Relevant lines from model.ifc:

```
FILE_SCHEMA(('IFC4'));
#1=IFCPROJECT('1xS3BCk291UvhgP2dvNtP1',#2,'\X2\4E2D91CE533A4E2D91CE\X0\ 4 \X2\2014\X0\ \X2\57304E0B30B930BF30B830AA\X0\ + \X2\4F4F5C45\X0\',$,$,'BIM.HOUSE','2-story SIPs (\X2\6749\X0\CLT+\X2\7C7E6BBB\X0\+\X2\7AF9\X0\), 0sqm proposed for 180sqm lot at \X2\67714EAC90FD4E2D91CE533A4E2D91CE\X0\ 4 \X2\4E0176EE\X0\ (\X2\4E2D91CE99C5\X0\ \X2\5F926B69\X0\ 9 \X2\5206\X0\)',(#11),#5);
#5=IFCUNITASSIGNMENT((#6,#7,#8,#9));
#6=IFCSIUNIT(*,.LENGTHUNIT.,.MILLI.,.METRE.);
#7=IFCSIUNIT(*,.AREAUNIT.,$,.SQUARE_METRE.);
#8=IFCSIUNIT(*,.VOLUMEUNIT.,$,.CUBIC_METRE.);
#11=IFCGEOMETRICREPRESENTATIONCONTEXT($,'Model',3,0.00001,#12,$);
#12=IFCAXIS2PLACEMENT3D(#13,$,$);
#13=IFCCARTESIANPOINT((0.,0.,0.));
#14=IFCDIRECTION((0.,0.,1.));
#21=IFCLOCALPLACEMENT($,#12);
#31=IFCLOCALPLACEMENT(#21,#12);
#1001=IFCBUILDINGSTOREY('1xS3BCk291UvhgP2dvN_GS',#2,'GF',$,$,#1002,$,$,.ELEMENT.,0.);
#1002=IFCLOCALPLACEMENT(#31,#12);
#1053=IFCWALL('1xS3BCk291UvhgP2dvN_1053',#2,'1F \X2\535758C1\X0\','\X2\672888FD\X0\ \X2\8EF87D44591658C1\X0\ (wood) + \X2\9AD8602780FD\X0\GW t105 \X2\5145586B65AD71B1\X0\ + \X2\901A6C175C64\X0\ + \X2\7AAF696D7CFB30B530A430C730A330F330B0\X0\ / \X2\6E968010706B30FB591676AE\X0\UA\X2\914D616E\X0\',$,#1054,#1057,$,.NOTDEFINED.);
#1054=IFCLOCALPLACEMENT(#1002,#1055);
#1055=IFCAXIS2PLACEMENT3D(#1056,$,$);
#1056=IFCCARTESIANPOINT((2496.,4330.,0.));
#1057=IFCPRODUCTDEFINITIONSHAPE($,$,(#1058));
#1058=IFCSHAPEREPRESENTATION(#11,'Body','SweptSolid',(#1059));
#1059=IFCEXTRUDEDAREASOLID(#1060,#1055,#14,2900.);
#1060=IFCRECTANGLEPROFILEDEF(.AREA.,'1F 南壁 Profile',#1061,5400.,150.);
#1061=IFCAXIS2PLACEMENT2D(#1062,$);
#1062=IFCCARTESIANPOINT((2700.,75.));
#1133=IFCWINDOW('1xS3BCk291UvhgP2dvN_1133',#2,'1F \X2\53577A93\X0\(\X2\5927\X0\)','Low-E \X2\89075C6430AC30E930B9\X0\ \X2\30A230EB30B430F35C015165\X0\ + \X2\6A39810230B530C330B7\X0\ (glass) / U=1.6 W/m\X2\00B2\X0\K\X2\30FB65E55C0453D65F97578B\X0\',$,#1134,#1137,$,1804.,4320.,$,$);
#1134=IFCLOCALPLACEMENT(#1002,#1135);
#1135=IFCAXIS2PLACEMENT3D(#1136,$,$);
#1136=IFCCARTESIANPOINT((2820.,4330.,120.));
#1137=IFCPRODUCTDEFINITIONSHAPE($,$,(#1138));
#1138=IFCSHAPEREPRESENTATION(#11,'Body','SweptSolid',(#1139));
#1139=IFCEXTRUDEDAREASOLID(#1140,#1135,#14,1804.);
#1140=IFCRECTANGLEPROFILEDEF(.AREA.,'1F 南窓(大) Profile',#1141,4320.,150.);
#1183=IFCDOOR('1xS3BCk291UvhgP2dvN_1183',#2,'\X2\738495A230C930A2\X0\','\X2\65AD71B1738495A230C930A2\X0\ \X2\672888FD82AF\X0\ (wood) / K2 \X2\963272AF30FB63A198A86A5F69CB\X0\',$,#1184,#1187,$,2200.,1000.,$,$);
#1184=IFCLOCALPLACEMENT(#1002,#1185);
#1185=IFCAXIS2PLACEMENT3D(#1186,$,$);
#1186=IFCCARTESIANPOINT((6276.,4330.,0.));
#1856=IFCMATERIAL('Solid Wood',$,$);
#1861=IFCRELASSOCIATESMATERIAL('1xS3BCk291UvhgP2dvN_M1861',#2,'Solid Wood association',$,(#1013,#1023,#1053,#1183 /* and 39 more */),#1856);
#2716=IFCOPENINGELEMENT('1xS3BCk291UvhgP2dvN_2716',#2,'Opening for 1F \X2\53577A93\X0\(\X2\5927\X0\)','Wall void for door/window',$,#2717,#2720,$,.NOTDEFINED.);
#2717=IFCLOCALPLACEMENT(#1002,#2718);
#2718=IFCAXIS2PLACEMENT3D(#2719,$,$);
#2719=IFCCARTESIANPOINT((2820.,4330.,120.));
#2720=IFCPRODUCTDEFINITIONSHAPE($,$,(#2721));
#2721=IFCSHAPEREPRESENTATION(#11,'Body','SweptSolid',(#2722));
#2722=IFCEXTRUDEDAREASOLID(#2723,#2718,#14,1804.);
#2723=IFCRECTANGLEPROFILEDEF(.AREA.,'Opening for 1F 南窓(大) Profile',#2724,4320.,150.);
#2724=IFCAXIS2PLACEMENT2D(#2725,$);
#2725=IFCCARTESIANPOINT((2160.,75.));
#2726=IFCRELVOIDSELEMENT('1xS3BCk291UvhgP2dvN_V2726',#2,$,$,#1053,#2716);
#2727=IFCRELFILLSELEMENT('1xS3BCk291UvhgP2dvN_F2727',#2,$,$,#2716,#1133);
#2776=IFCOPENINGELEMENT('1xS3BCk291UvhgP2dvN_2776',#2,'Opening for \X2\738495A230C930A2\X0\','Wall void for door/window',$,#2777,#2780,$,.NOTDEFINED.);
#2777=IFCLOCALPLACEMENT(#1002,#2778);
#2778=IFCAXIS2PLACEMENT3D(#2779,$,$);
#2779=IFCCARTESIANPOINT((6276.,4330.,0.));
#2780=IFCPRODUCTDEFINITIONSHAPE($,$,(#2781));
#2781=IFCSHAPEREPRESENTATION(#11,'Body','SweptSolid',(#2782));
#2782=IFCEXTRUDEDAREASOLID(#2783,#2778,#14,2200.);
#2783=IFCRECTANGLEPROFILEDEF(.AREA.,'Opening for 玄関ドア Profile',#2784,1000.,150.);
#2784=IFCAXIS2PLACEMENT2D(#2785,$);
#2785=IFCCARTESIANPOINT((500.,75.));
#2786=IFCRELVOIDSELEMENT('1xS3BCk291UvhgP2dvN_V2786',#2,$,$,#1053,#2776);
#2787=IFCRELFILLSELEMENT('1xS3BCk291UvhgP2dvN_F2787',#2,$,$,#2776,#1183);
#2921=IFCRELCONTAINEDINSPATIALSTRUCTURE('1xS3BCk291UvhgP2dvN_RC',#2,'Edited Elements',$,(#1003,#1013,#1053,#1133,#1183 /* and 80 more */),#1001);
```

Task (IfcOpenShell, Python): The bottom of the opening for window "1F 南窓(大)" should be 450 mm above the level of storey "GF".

```python
import numpy as np
import ifcopenshell
import ifcopenshell.api.geometry
import ifcopenshell.geom
import ifcopenshell.util.element
import ifcopenshell.util.placement
import ifcopenshell.util.shape
import ifcopenshell.util.unit

model = ifcopenshell.open("model.ifc")
unit_scale = ifcopenshell.util.unit.calculate_unit_scale(model)

window = model.by_guid("1xS3BCk291UvhgP2dvN_1133")
opening = window.FillsVoids[0].RelatingOpeningElement
storey = ifcopenshell.util.element.get_container(window, ifc_class="IfcBuildingStorey")
level = ifcopenshell.util.placement.get_local_placement(storey.ObjectPlacement)[2, 3]

# The opening's origin need not be at the sill, so measure its lowest point.
shape = ifcopenshell.geom.create_shape(ifcopenshell.geom.settings(), opening)
bottom = ifcopenshell.util.shape.get_shape_bottom_elevation(shape, shape.geometry) / unit_scale
dz = level + 450.0 - bottom

shift = np.array([0.0, 0.0, dz])
# The window is not placed relative to its opening, so move both.
for product in (opening, window):
    matrix = ifcopenshell.util.placement.get_local_placement(product.ObjectPlacement)
    matrix[:3, 3] += shift
    ifcopenshell.api.geometry.edit_object_placement(model, product=product, matrix=matrix, is_si=False)

print(f"moved by {dz * unit_scale:+.3f} m")

model.write("model-out.ifc")
```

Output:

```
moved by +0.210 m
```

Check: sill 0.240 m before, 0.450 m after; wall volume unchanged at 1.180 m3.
